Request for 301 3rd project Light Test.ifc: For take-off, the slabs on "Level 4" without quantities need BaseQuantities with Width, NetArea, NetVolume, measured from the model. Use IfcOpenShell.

First a look at what the model holds.

```python
import ifcopenshell
import ifcopenshell.util.element
import ifcopenshell.util.unit

model = ifcopenshell.open("301 3rd project Light Test.ifc")
print(model.schema)
for unit_type in ("LENGTHUNIT", "AREAUNIT", "VOLUMEUNIT"):
    print(unit_type, ifcopenshell.util.unit.calculate_unit_scale(model, unit_type))
storey = next(s for s in model.by_type("IfcBuildingStorey") if s.Name == "Level 4")
slabs = [e for e in ifcopenshell.util.element.get_decomposition(storey) if e.is_a("IfcSlab")]
for e in sorted(slabs, key=lambda e: e.id()):
    print(e.id(), e.is_a(), e.Name, list(ifcopenshell.util.element.get_psets(e, qtos_only=True)), sep=" | ")
```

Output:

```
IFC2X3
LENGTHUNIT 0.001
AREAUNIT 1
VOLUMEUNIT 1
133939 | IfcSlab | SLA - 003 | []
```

```python
import ifcopenshell
import ifcopenshell.api.pset
import ifcopenshell.geom
import ifcopenshell.util.element
import ifcopenshell.util.shape
import ifcopenshell.util.unit

model = ifcopenshell.open("301 3rd project Light Test.ifc")
unit_scale = ifcopenshell.util.unit.calculate_unit_scale(model)
area_scale = ifcopenshell.util.unit.calculate_unit_scale(model, "AREAUNIT")
volume_scale = ifcopenshell.util.unit.calculate_unit_scale(model, "VOLUMEUNIT")
settings = ifcopenshell.geom.settings()

storey = next(s for s in model.by_type("IfcBuildingStorey") if s.Name == "Level 4")
slabs = [e for e in ifcopenshell.util.element.get_decomposition(storey) if e.is_a("IfcSlab")]

for e in sorted(slabs, key=lambda e: e.id()):
    if ifcopenshell.util.element.get_psets(e, qtos_only=True, should_inherit=False):
        continue
    # Geometry comes back in metres, in the element's own axes.
    shape = ifcopenshell.geom.create_shape(settings, e)
    values = {
        "Width": ifcopenshell.util.shape.get_z(shape.geometry) / unit_scale,
        "NetArea": ifcopenshell.util.shape.get_footprint_area(shape.geometry) / area_scale,
        "NetVolume": ifcopenshell.util.shape.get_volume(shape.geometry) / volume_scale,
    }
    qto = ifcopenshell.api.pset.add_qto(model, product=e, name="BaseQuantities")
    ifcopenshell.api.pset.edit_qto(model, qto=qto, properties=values)
    print(e.id(), {k: round(v, 3) for k, v in values.items()})

model.write("301 3rd project Light Test_v2.ifc")
```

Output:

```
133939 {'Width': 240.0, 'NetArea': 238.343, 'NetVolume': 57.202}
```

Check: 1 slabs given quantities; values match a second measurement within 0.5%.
